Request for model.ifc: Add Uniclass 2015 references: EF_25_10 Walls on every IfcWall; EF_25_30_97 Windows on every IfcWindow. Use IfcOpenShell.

First a look at what the model holds.

```python
import ifcopenshell

model = ifcopenshell.open("model.ifc")
print(model.schema)
print("classifications:", [c.Name for c in model.by_type("IfcClassification")])
for ifc_class in ("IfcDoor", "IfcRoof", "IfcStair", "IfcWall", "IfcWindow"):
    print(ifc_class, len(model.by_type(ifc_class)))
```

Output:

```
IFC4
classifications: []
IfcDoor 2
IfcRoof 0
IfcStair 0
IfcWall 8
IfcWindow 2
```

```python
import ifcopenshell
import ifcopenshell.api.classification

model = ifcopenshell.open("model.ifc")

system = ifcopenshell.api.classification.add_classification(model, classification="Uniclass 2015")

codes = {
    "IfcWall": ("EF_25_10", "Walls"),
    "IfcWindow": ("EF_25_30_97", "Windows"),
}
for ifc_class, (code, name) in codes.items():
    products = model.by_type(ifc_class)
    ifcopenshell.api.classification.add_reference(
        model, products=products, classification=system, identification=code, name=name
    )
    print(code, len(products))

model.write("model_updated.ifc")
```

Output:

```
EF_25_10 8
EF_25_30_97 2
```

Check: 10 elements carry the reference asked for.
